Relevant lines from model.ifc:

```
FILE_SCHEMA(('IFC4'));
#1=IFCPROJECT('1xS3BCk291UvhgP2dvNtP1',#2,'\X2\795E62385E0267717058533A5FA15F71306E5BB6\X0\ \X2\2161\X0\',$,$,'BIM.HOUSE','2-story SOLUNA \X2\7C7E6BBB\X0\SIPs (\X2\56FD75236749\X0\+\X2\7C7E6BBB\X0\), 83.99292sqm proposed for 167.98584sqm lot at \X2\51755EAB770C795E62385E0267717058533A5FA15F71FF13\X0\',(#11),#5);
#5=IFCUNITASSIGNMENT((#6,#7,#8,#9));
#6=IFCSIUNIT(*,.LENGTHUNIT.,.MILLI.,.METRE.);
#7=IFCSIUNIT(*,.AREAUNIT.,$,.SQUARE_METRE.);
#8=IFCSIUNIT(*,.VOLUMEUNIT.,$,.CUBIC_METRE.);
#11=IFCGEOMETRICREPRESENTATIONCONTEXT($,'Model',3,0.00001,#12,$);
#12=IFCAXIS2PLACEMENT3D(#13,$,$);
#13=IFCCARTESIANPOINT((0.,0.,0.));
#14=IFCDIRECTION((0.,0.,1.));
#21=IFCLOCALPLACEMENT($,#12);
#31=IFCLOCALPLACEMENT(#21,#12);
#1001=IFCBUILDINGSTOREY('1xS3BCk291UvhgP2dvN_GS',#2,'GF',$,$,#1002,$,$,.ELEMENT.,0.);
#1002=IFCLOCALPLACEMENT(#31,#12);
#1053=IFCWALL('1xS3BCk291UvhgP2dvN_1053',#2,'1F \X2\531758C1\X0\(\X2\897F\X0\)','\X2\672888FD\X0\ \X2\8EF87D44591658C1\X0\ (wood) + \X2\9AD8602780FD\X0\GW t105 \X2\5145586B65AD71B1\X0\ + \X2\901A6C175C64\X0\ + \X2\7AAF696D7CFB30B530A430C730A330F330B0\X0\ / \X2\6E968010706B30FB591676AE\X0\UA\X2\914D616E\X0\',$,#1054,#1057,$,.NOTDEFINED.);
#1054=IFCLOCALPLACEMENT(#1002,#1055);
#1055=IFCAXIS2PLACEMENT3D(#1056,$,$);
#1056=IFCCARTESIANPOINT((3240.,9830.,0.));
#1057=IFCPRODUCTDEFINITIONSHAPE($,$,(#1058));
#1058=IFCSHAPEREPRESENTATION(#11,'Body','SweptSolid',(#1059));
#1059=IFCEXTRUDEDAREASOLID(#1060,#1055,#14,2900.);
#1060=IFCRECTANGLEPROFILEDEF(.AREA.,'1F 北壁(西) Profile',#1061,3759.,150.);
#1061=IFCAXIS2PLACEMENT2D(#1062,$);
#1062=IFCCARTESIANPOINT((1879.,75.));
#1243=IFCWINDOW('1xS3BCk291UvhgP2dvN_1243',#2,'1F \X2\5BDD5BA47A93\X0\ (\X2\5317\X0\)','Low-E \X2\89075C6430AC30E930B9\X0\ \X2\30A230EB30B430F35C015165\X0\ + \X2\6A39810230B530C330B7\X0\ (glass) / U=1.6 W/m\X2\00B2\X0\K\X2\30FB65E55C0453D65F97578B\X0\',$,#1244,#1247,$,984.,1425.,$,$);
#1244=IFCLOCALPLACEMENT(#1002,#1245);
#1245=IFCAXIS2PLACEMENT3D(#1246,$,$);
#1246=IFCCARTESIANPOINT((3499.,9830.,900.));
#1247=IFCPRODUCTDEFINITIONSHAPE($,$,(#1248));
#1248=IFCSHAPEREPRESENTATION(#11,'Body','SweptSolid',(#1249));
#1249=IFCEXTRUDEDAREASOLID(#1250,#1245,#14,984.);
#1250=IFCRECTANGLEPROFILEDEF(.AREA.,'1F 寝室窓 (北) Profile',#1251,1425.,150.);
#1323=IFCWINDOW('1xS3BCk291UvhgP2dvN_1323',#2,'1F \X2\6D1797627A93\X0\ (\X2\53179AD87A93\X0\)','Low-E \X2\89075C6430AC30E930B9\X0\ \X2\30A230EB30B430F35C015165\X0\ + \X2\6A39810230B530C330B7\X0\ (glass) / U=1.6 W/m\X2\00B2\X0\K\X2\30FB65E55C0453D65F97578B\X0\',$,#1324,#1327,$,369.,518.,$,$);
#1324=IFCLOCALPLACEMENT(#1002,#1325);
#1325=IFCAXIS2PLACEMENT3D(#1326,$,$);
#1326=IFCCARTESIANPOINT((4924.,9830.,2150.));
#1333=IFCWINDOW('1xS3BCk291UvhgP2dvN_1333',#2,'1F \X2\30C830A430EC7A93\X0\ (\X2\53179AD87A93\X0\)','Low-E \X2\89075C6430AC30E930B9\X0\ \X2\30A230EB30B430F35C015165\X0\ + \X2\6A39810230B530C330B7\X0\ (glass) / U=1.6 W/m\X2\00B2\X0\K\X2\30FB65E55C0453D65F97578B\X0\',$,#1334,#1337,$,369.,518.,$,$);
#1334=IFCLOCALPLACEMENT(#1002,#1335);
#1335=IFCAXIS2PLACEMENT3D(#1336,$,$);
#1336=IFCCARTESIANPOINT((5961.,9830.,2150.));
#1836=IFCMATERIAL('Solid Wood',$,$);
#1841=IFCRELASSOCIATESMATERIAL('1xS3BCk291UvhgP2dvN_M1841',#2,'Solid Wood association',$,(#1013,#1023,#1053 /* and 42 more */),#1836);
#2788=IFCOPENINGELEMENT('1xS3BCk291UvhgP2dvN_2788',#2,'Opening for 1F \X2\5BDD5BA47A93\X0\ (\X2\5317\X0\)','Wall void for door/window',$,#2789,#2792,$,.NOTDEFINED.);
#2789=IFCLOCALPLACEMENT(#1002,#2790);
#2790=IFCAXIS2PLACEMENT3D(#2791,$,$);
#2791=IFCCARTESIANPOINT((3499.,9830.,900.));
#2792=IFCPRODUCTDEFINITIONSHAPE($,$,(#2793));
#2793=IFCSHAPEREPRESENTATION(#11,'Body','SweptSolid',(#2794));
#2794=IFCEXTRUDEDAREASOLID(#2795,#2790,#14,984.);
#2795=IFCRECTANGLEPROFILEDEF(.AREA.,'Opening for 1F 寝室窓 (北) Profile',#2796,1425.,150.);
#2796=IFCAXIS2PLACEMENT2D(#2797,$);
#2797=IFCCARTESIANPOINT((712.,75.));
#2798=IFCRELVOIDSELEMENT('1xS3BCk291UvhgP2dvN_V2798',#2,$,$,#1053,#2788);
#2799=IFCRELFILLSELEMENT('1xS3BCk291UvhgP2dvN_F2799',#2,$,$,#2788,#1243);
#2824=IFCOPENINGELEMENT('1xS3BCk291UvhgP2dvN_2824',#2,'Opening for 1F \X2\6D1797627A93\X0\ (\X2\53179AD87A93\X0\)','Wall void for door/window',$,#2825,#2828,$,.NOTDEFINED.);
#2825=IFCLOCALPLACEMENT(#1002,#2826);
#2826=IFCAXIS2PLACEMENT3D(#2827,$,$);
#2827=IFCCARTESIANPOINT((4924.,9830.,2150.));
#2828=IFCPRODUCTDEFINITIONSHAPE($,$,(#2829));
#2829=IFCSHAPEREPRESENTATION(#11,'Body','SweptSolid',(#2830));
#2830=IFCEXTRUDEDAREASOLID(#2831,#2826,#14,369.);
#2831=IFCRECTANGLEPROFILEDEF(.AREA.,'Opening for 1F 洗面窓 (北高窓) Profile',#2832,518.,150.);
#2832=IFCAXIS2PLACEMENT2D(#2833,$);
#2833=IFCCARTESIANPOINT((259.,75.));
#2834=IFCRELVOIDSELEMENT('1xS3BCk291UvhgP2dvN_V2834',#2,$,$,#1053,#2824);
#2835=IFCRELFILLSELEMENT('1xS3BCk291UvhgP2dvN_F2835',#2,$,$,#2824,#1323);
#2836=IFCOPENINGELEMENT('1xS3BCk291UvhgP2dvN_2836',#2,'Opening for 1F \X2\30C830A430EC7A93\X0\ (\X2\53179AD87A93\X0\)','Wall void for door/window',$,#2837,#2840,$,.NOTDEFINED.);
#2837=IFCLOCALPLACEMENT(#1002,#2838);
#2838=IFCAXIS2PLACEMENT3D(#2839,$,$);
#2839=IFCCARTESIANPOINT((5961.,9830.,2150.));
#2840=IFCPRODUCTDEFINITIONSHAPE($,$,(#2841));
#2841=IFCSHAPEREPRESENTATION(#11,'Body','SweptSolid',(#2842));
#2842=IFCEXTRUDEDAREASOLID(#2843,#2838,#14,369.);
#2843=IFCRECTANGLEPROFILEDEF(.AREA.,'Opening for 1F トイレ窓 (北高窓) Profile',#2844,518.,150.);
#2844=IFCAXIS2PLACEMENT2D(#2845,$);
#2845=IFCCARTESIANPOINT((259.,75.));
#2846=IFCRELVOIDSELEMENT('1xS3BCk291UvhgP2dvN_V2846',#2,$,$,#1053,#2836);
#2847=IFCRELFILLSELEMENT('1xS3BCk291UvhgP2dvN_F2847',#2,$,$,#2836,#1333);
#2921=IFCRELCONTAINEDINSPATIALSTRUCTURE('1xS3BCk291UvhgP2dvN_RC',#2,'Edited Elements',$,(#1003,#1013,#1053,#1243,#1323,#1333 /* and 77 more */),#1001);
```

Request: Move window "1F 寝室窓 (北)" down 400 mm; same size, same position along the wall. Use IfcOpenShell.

```python
import numpy as np
import ifcopenshell
import ifcopenshell.api.geometry
import ifcopenshell.util.placement
import ifcopenshell.util.unit

model = ifcopenshell.open("model.ifc")
unit_scale = ifcopenshell.util.unit.calculate_unit_scale(model)

window = model.by_guid("1xS3BCk291UvhgP2dvN_1243")
opening = window.FillsVoids[0].RelatingOpeningElement
dz = -0.4 / unit_scale

shift = np.array([0.0, 0.0, dz])
# The window is not placed relative to its opening, so move both.
for product in (opening, window):
    matrix = ifcopenshell.util.placement.get_local_placement(product.ObjectPlacement)
    matrix[:3, 3] += shift
    ifcopenshell.api.geometry.edit_object_placement(model, product=product, matrix=matrix, is_si=False)

print(f"moved by {dz * unit_scale:+.3f} m")

model.write("model_rev.ifc")
```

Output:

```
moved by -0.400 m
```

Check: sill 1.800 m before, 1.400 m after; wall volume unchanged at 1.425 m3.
